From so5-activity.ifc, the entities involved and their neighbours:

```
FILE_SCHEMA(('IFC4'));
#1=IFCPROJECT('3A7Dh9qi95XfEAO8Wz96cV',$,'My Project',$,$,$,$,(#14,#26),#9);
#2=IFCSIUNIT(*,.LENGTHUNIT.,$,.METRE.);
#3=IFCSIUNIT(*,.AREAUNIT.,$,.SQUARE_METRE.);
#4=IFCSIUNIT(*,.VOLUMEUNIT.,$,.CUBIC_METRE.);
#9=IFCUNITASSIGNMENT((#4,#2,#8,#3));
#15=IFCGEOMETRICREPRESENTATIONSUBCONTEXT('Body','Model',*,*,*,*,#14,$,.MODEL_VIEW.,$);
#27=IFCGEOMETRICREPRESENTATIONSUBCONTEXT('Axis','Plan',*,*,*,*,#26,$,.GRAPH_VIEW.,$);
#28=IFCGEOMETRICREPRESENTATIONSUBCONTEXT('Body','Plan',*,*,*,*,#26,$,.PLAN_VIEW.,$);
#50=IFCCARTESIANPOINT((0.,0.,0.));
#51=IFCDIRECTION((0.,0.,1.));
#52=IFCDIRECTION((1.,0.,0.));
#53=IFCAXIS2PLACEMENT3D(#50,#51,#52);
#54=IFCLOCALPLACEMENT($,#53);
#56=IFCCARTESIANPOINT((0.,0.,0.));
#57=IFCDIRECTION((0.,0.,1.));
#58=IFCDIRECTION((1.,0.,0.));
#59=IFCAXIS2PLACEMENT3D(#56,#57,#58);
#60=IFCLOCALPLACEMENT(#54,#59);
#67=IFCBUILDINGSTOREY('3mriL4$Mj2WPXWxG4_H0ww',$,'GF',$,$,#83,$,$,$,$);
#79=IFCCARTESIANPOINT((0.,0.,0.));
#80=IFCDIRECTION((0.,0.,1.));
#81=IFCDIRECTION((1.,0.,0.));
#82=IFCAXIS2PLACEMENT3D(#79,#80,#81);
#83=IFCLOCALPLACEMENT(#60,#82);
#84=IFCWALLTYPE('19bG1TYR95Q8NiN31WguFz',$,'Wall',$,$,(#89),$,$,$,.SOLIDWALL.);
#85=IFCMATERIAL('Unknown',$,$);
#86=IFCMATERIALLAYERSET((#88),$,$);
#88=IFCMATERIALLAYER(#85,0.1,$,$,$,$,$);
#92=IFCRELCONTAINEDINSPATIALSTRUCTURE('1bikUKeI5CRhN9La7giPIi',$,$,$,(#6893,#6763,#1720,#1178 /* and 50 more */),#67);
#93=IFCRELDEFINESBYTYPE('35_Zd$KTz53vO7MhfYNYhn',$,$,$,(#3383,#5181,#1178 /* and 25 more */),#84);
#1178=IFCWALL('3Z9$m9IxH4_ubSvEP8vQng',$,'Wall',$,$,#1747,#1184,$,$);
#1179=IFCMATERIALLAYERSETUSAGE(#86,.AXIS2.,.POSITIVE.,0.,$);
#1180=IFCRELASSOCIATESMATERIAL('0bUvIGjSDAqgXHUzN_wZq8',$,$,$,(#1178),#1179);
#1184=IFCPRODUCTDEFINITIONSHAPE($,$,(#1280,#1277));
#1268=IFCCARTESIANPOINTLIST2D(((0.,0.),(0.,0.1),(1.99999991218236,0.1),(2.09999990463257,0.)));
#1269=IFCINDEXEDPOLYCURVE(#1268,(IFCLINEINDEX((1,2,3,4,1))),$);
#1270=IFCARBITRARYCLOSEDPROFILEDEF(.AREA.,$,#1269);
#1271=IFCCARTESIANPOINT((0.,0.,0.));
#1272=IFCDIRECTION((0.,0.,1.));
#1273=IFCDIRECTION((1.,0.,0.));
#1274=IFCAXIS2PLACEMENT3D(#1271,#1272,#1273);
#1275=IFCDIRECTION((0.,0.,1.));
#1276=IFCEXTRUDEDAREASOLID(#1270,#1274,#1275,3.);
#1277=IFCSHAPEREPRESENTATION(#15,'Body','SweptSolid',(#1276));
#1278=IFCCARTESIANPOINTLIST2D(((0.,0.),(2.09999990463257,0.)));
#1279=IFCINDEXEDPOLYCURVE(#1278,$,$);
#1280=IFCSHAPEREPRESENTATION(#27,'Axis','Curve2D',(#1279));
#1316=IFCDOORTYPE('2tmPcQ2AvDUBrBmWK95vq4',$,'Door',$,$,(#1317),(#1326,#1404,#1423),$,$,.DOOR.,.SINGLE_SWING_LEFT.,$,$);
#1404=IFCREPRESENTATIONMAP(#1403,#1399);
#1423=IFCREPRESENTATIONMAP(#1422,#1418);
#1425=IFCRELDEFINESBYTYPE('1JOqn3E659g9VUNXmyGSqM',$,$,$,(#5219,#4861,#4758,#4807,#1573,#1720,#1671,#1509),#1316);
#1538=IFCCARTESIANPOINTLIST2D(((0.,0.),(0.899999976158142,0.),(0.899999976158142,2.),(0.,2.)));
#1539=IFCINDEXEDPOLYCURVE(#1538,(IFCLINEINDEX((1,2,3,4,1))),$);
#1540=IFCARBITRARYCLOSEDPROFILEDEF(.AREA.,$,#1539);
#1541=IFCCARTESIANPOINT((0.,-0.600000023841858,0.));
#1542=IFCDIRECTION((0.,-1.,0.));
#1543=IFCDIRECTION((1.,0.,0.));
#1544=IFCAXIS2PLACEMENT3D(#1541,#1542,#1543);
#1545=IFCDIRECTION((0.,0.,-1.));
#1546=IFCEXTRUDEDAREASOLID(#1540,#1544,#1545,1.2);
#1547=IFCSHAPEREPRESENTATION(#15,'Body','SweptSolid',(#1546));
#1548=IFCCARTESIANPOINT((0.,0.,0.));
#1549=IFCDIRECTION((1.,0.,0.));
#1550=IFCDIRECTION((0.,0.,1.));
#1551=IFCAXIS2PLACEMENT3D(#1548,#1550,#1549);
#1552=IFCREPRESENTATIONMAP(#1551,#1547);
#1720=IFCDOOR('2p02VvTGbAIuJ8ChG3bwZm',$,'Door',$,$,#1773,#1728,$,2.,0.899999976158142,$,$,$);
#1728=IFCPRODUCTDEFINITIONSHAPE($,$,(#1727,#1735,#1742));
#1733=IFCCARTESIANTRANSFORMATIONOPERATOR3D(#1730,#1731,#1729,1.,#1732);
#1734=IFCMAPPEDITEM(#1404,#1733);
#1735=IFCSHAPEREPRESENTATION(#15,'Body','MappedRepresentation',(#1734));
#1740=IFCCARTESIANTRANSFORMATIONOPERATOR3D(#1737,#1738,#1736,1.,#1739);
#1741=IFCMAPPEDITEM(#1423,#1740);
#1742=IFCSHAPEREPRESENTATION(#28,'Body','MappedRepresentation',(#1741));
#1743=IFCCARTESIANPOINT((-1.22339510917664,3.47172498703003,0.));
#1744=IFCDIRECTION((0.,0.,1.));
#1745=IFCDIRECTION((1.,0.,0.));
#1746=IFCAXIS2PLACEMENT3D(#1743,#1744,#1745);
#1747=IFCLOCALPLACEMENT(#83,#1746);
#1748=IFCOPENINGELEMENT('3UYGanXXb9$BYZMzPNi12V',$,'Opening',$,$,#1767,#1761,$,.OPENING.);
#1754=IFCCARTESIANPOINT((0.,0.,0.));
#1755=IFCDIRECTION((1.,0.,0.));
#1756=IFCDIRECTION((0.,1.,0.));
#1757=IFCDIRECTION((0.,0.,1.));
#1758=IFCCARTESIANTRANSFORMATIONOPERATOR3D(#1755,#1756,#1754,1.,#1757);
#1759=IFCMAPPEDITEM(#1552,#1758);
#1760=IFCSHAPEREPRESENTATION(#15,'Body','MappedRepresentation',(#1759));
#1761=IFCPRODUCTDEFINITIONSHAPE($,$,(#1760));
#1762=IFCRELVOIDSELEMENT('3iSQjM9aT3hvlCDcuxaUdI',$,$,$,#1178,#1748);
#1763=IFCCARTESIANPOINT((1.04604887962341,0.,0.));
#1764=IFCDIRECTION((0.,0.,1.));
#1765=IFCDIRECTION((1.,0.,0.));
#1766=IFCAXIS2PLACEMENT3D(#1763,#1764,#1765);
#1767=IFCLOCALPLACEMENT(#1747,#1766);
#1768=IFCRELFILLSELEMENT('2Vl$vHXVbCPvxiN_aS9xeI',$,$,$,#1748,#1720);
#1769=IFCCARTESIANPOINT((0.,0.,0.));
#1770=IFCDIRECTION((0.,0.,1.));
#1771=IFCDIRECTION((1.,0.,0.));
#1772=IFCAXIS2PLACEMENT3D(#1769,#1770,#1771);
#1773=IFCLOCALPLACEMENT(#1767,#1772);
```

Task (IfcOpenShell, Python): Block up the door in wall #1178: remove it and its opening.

```python
import ifcopenshell
import ifcopenshell.api.feature
import ifcopenshell.api.root
import ifcopenshell.geom
import ifcopenshell.util.shape

model = ifcopenshell.open("so5-activity.ifc")
settings = ifcopenshell.geom.settings()


def volume(element):
    """Net volume in cubic metres, openings subtracted."""
    shape = ifcopenshell.geom.create_shape(settings, element)
    return ifcopenshell.util.shape.get_volume(shape.geometry)


door = model.by_guid("2p02VvTGbAIuJ8ChG3bwZm")
opening = door.FillsVoids[0].RelatingOpeningElement
wall = opening.VoidsElements[0].RelatingBuildingElement
before = volume(wall)

ifcopenshell.api.root.remove_product(model, product=door)
ifcopenshell.api.feature.remove_feature(model, feature=opening)

after = volume(wall)

print(f"wall volume {before:.3f} -> {after:.3f} m3")

model.write("so5-activity_rev.ifc")
```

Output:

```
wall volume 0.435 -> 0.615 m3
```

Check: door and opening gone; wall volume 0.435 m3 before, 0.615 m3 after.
